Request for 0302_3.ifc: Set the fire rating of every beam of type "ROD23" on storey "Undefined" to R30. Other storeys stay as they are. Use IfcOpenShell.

First a look at what the model holds.

```python
import ifcopenshell
import ifcopenshell.util.element

model = ifcopenshell.open("0302_3.ifc")
print(model.schema)
storey = next(s for s in model.by_type("IfcBuildingStorey") if s.Name == "Undefined")
beams = [e for e in ifcopenshell.util.element.get_decomposition(storey) if e.is_a("IfcBeam")]
seen = {}
for e in beams:
    element_type = ifcopenshell.util.element.get_type(e)
    key = (element_type.Name if element_type != e and element_type else None, ifcopenshell.util.element.get_pset(e, "Pset_BeamCommon", "FireRating"))
    seen[key] = seen.get(key, 0) + 1
for (name, value), count in sorted(seen.items(), key=str):
    print(count, "x", name, "|", value)
```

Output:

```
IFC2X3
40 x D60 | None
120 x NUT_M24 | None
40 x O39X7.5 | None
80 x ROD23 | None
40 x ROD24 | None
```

```python
import ifcopenshell
import ifcopenshell.api.pset
import ifcopenshell.util.element

model = ifcopenshell.open("0302_3.ifc")

storey = next(s for s in model.by_type("IfcBuildingStorey") if s.Name == "Undefined")
beams = [e for e in ifcopenshell.util.element.get_decomposition(storey) if e.is_a("IfcBeam")]

count = 0
for e in beams:
    element_type = ifcopenshell.util.element.get_type(e)
    if element_type in (None, e) or element_type.Name != "ROD23":
        continue
    found = ifcopenshell.util.element.get_pset(e, "Pset_BeamCommon", should_inherit=False)
    if found:
        pset = model.by_id(found["id"])
        if len(ifcopenshell.util.element.get_elements_by_pset(pset)) > 1:
            pset = ifcopenshell.api.pset.unshare_pset(model, products=[e], pset=pset)[0]
    else:
        pset = ifcopenshell.api.pset.add_pset(model, product=e, name="Pset_BeamCommon")
    ifcopenshell.api.pset.edit_pset(model, pset=pset, properties={"FireRating": "R30"})
    count += 1

print(count, "beams updated")

model.write("0302_3_edited.ifc")
```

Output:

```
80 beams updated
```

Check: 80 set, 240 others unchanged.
